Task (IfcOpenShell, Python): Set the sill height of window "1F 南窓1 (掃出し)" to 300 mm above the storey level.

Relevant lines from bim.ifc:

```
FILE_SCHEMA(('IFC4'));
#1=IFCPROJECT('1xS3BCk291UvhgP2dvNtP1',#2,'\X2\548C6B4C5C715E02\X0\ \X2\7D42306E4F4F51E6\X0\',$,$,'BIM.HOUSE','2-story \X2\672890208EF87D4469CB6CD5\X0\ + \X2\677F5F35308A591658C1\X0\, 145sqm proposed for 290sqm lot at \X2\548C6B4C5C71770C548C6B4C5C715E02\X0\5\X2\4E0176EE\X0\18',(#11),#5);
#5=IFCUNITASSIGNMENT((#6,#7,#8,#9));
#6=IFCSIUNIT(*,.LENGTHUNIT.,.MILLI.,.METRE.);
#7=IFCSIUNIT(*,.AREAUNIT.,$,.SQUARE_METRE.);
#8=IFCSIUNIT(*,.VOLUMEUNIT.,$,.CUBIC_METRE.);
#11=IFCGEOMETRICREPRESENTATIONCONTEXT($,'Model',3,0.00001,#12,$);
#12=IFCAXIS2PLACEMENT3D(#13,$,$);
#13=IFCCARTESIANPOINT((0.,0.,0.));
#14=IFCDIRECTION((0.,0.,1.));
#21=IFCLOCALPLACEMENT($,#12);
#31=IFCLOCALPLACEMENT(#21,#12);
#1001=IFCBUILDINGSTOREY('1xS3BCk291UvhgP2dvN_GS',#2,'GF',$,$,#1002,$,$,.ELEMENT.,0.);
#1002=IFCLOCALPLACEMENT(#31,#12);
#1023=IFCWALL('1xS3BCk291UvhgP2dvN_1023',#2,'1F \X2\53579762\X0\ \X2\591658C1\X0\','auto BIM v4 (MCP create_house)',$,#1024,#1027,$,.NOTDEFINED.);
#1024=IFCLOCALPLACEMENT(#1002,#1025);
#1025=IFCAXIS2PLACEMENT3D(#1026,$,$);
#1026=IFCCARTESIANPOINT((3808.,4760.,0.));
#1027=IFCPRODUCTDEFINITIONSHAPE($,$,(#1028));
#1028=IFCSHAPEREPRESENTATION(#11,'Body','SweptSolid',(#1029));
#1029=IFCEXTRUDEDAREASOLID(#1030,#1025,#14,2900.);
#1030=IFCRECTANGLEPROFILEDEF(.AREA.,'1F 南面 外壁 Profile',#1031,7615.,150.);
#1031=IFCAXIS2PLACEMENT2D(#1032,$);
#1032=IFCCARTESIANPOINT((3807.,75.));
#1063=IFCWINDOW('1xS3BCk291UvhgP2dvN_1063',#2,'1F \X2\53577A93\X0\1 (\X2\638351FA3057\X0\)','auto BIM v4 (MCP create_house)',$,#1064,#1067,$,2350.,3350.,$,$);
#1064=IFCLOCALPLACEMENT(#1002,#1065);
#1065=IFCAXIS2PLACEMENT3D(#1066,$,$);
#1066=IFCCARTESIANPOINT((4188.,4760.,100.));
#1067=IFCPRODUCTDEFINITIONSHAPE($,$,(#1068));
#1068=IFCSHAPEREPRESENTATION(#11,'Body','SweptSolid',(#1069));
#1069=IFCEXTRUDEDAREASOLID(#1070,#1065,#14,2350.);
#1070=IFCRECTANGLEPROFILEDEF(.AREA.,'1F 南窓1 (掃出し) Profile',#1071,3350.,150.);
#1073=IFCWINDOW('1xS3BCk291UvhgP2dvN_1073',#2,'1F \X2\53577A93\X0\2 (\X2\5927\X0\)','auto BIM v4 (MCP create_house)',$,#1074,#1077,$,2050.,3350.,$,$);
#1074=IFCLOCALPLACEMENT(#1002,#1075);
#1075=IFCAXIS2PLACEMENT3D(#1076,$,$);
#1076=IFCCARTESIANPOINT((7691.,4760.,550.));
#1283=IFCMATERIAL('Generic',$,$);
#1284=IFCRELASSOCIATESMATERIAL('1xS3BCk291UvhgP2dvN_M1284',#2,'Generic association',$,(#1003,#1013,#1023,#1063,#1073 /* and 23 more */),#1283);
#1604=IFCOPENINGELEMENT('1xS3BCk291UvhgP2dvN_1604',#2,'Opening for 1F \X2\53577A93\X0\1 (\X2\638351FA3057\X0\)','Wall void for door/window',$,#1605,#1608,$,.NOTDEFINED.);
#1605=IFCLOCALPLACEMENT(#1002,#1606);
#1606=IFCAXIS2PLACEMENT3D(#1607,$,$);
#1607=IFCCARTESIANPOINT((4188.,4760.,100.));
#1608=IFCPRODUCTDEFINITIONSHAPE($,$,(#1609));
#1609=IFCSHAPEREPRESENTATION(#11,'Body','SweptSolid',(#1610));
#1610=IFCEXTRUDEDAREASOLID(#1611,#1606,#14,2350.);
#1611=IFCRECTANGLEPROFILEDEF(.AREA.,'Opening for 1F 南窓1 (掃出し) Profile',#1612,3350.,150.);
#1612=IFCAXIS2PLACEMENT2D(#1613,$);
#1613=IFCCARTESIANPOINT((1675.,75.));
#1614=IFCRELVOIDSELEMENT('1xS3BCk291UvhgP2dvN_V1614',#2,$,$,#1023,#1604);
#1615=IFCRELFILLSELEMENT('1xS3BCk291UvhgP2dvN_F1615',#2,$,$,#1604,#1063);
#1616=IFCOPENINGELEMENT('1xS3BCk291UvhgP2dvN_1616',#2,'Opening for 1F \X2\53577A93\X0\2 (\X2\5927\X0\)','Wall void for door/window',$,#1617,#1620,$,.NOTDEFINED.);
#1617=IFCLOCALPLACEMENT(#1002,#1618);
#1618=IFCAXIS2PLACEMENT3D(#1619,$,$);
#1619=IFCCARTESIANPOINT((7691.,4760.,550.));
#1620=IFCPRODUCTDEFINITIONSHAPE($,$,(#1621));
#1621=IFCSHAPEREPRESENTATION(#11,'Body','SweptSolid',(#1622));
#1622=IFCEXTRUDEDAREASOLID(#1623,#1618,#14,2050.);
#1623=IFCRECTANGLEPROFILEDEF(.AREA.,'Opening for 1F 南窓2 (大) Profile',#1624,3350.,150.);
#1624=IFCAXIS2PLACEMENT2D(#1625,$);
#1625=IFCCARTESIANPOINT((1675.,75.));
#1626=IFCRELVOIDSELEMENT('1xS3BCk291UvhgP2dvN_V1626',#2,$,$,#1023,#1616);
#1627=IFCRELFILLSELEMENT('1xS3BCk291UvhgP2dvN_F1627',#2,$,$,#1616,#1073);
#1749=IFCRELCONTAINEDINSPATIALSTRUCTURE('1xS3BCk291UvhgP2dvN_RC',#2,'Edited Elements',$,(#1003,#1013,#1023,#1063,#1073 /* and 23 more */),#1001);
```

```python
import numpy as np
import ifcopenshell
import ifcopenshell.api.geometry
import ifcopenshell.geom
import ifcopenshell.util.element
import ifcopenshell.util.placement
import ifcopenshell.util.shape
import ifcopenshell.util.unit

model = ifcopenshell.open("bim.ifc")
unit_scale = ifcopenshell.util.unit.calculate_unit_scale(model)

window = model.by_guid("1xS3BCk291UvhgP2dvN_1063")
opening = window.FillsVoids[0].RelatingOpeningElement
storey = ifcopenshell.util.element.get_container(window, ifc_class="IfcBuildingStorey")
level = ifcopenshell.util.placement.get_local_placement(storey.ObjectPlacement)[2, 3]

# The opening's origin need not be at the sill, so measure its lowest point.
shape = ifcopenshell.geom.create_shape(ifcopenshell.geom.settings(), opening)
bottom = ifcopenshell.util.shape.get_shape_bottom_elevation(shape, shape.geometry) / unit_scale
dz = level + 0.3 / unit_scale - bottom

shift = np.array([0.0, 0.0, dz])
# The window is not placed relative to its opening, so move both.
for product in (opening, window):
    matrix = ifcopenshell.util.placement.get_local_placement(product.ObjectPlacement)
    matrix[:3, 3] += shift
    ifcopenshell.api.geometry.edit_object_placement(model, product=product, matrix=matrix, is_si=False)

print(f"moved by {dz * unit_scale:+.3f} m")

model.write("bim-out.ifc")
```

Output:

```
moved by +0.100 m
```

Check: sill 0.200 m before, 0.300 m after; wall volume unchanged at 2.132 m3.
